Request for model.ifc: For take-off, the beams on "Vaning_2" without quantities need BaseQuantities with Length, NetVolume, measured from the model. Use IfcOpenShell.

First a look at what the model holds.

```python
import ifcopenshell
import ifcopenshell.util.element
import ifcopenshell.util.unit

model = ifcopenshell.open("model.ifc")
print(model.schema)
for unit_type in ("LENGTHUNIT", "AREAUNIT", "VOLUMEUNIT"):
    print(unit_type, ifcopenshell.util.unit.calculate_unit_scale(model, unit_type))
storey = next(s for s in model.by_type("IfcBuildingStorey") if s.Name == "Vaning_2")
beams = [e for e in ifcopenshell.util.element.get_decomposition(storey) if e.is_a("IfcBeam")]
for e in sorted(beams, key=lambda e: e.id()):
    print(e.id(), e.is_a(), e.Name, list(ifcopenshell.util.element.get_psets(e, qtos_only=True)), sep=" | ")
```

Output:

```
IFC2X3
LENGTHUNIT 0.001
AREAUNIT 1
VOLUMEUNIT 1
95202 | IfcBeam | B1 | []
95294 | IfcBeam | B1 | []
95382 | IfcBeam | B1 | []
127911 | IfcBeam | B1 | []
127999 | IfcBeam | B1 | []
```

```python
import ifcopenshell
import ifcopenshell.api.pset
import ifcopenshell.geom
import ifcopenshell.util.element
import ifcopenshell.util.shape
import ifcopenshell.util.unit

model = ifcopenshell.open("model.ifc")
unit_scale = ifcopenshell.util.unit.calculate_unit_scale(model)
volume_scale = ifcopenshell.util.unit.calculate_unit_scale(model, "VOLUMEUNIT")
settings = ifcopenshell.geom.settings()

storey = next(s for s in model.by_type("IfcBuildingStorey") if s.Name == "Vaning_2")
beams = [e for e in ifcopenshell.util.element.get_decomposition(storey) if e.is_a("IfcBeam")]

for e in sorted(beams, key=lambda e: e.id()):
    if ifcopenshell.util.element.get_psets(e, qtos_only=True, should_inherit=False):
        continue
    # Geometry comes back in metres, in the element's own axes.
    shape = ifcopenshell.geom.create_shape(settings, e)
    values = {
        "Length": ifcopenshell.util.shape.get_max_xyz(shape.geometry) / unit_scale,
        "NetVolume": ifcopenshell.util.shape.get_volume(shape.geometry) / volume_scale,
    }
    qto = ifcopenshell.api.pset.add_qto(model, product=e, name="BaseQuantities")
    ifcopenshell.api.pset.edit_qto(model, qto=qto, properties=values)
    print(e.id(), {k: round(v, 3) for k, v in values.items()})

model.write("model_updated.ifc")
```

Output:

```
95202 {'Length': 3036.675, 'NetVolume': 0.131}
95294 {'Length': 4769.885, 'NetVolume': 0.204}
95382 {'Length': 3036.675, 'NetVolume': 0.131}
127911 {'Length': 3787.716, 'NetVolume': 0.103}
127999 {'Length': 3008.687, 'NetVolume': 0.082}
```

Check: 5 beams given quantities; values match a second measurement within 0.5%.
